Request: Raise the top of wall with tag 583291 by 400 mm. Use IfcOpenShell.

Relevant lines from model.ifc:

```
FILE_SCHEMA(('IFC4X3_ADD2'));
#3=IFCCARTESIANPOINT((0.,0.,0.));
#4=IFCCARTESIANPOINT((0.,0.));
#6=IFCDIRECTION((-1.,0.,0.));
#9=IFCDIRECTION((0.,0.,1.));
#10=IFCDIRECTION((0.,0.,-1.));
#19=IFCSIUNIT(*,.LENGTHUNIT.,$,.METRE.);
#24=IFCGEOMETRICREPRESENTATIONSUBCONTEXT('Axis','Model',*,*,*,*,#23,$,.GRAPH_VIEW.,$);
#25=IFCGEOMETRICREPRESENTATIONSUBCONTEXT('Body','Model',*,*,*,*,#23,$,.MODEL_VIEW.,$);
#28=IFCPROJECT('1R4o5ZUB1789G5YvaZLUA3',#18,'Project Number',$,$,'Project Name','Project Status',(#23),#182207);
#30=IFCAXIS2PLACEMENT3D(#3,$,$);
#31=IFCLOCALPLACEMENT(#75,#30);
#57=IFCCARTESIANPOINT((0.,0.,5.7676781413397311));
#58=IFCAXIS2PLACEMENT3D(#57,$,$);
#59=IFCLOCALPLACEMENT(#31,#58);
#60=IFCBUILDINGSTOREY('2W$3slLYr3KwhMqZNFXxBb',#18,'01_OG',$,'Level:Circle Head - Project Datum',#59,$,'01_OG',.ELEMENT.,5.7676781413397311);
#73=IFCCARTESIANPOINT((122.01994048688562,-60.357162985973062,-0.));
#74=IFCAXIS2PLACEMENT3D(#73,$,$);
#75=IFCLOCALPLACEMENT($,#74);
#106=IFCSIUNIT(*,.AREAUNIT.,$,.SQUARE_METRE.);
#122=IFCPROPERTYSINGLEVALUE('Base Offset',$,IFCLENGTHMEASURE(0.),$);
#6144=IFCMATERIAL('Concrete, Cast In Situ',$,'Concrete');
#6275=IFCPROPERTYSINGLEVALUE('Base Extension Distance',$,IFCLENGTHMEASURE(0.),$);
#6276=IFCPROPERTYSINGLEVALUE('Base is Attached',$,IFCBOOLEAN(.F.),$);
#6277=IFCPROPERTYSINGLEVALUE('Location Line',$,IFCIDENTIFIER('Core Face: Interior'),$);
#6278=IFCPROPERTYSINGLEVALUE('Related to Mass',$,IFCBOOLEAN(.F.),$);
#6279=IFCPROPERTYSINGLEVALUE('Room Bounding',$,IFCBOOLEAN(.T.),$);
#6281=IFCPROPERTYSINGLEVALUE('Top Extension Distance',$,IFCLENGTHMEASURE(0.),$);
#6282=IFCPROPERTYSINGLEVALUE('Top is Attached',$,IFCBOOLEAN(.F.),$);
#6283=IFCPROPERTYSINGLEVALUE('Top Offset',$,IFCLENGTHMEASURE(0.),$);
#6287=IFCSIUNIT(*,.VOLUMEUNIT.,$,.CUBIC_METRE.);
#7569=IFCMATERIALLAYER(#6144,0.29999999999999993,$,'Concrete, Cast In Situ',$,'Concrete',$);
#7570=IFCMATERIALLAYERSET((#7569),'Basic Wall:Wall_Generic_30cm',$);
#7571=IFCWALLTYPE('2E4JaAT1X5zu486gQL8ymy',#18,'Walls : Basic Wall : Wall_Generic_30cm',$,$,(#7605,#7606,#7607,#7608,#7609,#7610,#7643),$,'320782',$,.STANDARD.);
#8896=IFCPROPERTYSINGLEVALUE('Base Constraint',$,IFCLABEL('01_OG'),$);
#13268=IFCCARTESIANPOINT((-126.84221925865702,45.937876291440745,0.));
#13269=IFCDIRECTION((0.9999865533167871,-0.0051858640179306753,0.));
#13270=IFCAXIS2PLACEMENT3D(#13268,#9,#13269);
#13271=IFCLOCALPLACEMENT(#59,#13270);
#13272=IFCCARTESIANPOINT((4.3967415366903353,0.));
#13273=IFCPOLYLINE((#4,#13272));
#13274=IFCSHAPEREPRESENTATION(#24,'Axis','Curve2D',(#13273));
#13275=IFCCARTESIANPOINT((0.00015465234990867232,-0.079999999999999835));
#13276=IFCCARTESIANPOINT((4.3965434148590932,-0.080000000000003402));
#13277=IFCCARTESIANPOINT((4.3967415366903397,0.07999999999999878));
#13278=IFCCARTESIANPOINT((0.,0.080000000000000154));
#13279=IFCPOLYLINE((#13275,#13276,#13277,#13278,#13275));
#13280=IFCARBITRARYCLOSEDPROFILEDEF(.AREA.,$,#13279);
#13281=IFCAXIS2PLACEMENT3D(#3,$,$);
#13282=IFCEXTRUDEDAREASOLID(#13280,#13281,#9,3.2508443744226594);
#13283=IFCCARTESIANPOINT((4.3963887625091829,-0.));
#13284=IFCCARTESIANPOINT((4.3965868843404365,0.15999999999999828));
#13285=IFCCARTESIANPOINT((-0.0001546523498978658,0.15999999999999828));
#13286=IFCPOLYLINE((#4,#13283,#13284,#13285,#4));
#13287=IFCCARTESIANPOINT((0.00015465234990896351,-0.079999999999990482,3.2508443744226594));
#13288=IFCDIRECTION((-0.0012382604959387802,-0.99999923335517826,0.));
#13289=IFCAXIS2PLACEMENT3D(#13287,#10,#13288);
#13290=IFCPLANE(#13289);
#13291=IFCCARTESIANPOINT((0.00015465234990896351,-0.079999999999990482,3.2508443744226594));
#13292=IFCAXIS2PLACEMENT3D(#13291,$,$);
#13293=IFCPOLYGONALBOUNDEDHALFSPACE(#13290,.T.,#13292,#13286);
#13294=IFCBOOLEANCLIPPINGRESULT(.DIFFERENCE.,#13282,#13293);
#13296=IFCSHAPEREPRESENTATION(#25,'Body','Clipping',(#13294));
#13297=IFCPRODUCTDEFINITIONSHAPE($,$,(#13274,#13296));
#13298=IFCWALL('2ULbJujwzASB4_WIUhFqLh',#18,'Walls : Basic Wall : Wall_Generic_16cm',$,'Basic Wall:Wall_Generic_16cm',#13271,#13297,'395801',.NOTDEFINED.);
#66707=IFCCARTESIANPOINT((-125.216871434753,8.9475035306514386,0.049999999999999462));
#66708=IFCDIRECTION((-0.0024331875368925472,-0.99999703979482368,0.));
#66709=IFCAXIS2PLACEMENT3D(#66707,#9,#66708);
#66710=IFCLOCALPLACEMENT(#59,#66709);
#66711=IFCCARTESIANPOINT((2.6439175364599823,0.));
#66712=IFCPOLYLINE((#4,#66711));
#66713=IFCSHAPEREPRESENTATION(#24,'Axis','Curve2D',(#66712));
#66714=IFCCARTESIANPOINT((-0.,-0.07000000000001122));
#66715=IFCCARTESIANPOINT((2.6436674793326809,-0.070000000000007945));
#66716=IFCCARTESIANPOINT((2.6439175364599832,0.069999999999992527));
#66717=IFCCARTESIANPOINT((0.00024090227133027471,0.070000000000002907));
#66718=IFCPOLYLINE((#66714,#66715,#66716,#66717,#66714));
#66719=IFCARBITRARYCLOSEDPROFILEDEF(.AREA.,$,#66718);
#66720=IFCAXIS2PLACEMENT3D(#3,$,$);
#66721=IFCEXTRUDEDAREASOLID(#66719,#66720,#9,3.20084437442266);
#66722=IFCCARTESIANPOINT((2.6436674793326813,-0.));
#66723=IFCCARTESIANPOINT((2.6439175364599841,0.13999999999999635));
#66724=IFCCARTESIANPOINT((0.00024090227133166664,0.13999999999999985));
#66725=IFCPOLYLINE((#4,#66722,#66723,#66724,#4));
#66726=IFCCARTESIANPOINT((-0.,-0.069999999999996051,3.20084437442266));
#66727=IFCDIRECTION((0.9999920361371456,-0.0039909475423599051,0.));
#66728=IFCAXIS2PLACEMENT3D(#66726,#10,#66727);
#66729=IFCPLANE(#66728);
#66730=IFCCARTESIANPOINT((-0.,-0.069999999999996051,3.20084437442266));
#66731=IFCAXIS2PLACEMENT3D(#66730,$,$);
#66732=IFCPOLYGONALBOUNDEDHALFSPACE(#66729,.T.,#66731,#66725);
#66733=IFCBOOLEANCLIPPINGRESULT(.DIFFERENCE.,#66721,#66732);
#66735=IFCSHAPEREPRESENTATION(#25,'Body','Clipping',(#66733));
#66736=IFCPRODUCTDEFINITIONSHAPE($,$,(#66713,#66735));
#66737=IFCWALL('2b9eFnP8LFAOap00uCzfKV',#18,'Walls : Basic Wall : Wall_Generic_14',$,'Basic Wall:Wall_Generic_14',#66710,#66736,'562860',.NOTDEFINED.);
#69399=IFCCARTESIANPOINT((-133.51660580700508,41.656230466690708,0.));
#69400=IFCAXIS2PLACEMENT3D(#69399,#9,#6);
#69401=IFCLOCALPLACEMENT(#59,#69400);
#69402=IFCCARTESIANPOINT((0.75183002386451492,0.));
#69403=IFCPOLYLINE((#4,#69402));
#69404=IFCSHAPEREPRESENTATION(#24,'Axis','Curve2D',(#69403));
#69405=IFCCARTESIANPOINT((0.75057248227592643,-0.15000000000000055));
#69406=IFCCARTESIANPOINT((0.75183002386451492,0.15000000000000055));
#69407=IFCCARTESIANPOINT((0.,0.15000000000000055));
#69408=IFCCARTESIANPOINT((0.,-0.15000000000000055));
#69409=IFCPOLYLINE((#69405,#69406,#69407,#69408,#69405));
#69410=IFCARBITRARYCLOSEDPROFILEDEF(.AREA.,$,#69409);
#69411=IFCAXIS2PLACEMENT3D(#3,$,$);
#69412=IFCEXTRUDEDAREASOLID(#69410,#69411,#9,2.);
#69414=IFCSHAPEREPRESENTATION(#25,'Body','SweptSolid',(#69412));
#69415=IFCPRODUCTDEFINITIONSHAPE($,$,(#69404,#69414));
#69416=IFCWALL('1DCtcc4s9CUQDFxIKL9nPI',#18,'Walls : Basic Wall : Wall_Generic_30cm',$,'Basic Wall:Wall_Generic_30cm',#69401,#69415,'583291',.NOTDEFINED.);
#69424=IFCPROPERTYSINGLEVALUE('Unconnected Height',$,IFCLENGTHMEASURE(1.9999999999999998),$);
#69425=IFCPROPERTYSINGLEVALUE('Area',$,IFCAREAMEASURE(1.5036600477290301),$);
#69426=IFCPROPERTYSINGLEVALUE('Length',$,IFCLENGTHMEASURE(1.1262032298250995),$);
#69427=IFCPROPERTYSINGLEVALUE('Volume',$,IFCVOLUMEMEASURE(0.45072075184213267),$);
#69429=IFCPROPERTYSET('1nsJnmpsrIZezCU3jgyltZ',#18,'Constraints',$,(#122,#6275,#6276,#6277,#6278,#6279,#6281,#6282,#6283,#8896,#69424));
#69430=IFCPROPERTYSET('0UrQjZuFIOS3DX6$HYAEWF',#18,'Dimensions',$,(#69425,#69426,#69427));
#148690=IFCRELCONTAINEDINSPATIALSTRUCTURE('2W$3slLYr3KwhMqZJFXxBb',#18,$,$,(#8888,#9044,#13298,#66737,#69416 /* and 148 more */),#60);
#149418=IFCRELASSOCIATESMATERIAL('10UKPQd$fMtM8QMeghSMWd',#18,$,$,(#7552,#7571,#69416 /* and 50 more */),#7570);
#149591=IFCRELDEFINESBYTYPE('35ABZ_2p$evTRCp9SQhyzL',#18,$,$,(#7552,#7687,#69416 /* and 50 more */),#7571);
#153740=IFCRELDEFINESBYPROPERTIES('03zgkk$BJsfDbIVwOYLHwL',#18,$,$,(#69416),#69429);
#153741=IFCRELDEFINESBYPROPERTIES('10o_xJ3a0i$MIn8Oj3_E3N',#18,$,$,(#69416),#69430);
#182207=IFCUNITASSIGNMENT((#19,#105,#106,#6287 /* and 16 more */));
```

```python
import ifcopenshell
import ifcopenshell.api.pset
import ifcopenshell.geom
import ifcopenshell.util.element
import ifcopenshell.util.representation
import ifcopenshell.util.shape
import ifcopenshell.util.unit

model = ifcopenshell.open("model.ifc")
unit_scale = ifcopenshell.util.unit.calculate_unit_scale(model)
area_scale = ifcopenshell.util.unit.calculate_unit_scale(model, "AREAUNIT")
volume_scale = ifcopenshell.util.unit.calculate_unit_scale(model, "VOLUMEUNIT")
settings = ifcopenshell.geom.settings()


def volume(element):
    """Net volume in cubic metres, openings subtracted."""
    shape = ifcopenshell.geom.create_shape(settings, element)
    return ifcopenshell.util.shape.get_volume(shape.geometry)


wall = model.by_id(69416)
before = volume(wall)

body = ifcopenshell.util.representation.get_representation(wall, "Model", "Body")
solid = body.Items[0]
old_height = solid.Depth
solid.Depth += 0.4 / unit_scale
after = volume(wall)
thickness = 0.3  # wall thickness in metres

# Update the stored height, areas and volumes.
pset = model.by_id(ifcopenshell.util.element.get_pset(wall, "Constraints", should_inherit=False)["id"])
ifcopenshell.api.pset.edit_pset(model, pset=pset, properties={
    "Unconnected Height": model.create_entity("IfcLengthMeasure", solid.Depth),
})
pset = model.by_id(ifcopenshell.util.element.get_pset(wall, "Dimensions", should_inherit=False)["id"])
ifcopenshell.api.pset.edit_pset(model, pset=pset, properties={
    "Area": model.create_entity("IfcAreaMeasure", after / thickness / area_scale),
    "Volume": model.create_entity("IfcVolumeMeasure", after / volume_scale),
})

print(f"height {old_height:g} -> {solid.Depth:g}, volume {before:.3f} -> {after:.3f} m3")

model.write("model-out.ifc")
```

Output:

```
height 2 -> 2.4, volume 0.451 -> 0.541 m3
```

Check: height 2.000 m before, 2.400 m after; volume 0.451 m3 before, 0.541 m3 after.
